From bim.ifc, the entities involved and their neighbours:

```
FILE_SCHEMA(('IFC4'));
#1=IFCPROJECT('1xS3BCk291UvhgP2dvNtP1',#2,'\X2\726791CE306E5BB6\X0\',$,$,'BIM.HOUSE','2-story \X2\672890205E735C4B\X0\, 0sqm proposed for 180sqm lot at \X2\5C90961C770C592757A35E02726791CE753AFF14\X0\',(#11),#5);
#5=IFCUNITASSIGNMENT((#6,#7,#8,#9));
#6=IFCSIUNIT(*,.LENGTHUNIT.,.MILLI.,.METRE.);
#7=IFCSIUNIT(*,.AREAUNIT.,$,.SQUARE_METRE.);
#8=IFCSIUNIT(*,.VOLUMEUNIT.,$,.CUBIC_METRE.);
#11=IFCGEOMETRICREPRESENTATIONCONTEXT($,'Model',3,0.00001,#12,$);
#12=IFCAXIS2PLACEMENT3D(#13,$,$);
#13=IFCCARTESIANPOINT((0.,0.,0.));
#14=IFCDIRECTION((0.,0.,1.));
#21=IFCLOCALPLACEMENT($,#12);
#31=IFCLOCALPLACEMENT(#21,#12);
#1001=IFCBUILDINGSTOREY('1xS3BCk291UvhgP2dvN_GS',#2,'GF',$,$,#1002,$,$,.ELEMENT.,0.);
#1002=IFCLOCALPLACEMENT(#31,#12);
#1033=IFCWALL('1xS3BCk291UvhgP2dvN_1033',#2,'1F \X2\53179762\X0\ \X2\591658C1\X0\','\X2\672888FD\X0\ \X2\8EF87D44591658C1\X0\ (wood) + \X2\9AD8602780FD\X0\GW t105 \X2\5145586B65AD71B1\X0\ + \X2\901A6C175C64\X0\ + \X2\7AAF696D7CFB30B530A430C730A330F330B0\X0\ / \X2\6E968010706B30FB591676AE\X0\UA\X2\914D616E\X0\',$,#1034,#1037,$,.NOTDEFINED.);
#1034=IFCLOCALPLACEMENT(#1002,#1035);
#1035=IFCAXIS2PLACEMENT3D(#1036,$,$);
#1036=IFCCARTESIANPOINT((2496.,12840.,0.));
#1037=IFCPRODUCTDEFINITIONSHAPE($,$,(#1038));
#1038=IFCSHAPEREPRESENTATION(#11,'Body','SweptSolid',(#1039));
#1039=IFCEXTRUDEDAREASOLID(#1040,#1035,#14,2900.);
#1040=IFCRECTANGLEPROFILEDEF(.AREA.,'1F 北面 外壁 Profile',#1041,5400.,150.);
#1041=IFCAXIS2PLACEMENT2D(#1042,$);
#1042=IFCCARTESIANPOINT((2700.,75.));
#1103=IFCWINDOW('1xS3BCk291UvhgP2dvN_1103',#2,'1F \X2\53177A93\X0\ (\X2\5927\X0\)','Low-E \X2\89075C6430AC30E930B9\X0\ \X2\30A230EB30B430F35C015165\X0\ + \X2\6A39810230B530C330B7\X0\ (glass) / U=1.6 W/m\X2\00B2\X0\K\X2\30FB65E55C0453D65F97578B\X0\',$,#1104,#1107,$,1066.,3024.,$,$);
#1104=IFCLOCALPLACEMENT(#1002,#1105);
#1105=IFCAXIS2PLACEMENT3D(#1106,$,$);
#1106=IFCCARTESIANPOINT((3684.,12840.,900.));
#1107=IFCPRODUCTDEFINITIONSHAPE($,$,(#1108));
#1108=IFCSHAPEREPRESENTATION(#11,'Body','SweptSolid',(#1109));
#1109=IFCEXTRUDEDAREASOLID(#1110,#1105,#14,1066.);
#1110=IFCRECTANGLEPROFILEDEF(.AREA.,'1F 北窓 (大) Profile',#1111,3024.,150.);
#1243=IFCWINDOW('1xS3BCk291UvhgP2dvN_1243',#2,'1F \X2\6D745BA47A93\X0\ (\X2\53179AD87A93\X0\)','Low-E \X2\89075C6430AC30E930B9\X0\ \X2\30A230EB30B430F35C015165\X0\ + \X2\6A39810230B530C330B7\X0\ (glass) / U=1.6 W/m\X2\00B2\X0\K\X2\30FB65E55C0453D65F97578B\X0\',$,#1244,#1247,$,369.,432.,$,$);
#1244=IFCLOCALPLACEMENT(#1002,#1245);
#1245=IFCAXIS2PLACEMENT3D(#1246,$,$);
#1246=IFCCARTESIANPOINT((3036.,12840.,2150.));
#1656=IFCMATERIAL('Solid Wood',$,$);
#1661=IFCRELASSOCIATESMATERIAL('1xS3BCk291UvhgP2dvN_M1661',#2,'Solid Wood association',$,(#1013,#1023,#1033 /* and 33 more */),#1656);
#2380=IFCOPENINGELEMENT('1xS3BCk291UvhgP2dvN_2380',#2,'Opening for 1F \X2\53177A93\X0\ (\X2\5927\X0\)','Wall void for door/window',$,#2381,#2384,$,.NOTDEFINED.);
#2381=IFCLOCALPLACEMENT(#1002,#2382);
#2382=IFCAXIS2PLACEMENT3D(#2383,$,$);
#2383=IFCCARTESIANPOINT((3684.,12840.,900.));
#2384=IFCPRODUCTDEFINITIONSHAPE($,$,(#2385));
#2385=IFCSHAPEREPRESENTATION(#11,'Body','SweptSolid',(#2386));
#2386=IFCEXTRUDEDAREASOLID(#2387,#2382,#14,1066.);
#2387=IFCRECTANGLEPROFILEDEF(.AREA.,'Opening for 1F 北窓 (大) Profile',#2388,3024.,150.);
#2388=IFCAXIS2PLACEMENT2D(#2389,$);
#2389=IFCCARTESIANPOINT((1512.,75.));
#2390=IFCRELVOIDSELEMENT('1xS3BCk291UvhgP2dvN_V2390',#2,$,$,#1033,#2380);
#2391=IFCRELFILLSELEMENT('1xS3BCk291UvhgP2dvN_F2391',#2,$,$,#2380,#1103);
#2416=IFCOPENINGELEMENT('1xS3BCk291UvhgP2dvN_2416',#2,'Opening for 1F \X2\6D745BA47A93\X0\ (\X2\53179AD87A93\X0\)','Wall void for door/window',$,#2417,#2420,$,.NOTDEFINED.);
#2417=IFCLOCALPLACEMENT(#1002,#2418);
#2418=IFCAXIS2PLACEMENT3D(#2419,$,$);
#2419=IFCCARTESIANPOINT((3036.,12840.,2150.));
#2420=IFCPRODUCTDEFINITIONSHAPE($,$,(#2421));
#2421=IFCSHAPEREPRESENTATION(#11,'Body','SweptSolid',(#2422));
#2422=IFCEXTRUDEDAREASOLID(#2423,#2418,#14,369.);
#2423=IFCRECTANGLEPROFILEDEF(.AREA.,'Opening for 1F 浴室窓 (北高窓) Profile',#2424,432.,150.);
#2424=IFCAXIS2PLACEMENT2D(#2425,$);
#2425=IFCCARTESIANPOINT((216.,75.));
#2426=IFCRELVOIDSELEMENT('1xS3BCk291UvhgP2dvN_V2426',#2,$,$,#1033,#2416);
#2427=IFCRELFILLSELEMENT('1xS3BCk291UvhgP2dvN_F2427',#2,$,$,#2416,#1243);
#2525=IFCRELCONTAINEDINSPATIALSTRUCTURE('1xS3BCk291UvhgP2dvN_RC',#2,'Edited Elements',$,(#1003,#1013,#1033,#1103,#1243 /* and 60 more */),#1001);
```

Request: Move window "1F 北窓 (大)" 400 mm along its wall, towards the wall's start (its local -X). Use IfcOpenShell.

```python
import ifcopenshell
import ifcopenshell.api.geometry
import ifcopenshell.util.placement
import ifcopenshell.util.unit

model = ifcopenshell.open("bim.ifc")
unit_scale = ifcopenshell.util.unit.calculate_unit_scale(model)

window = model.by_guid("1xS3BCk291UvhgP2dvN_1103")
opening = window.FillsVoids[0].RelatingOpeningElement
wall = opening.VoidsElements[0].RelatingBuildingElement

wall_matrix = ifcopenshell.util.placement.get_local_placement(wall.ObjectPlacement)
shift = wall_matrix[:3, 0] * -0.4 / unit_scale
before = ifcopenshell.util.placement.get_local_placement(window.ObjectPlacement)[:3, 3].copy()

# The window is not placed relative to its opening, so move both.
for product in (opening, window):
    matrix = ifcopenshell.util.placement.get_local_placement(product.ObjectPlacement)
    matrix[:3, 3] += shift
    ifcopenshell.api.geometry.edit_object_placement(model, product=product, matrix=matrix, is_si=False)

after = ifcopenshell.util.placement.get_local_placement(window.ObjectPlacement)[:3, 3]
print("window moved by", (after - before).round(3) + 0.0)

model.write("bim_edited.ifc")
```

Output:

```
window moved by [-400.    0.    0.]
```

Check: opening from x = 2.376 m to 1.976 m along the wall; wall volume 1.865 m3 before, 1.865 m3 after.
